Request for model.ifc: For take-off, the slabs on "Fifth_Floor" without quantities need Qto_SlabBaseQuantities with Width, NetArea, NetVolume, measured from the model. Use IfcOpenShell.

First a look at what the model holds.

```python
import ifcopenshell
import ifcopenshell.util.element
import ifcopenshell.util.unit

model = ifcopenshell.open("model.ifc")
print(model.schema)
for unit_type in ("LENGTHUNIT", "AREAUNIT", "VOLUMEUNIT"):
    print(unit_type, ifcopenshell.util.unit.calculate_unit_scale(model, unit_type))
storey = next(s for s in model.by_type("IfcBuildingStorey") if s.Name == "Fifth_Floor")
slabs = [e for e in ifcopenshell.util.element.get_decomposition(storey) if e.is_a("IfcSlab")]
for e in sorted(slabs, key=lambda e: e.id()):
    print(e.id(), e.is_a(), e.Name, list(ifcopenshell.util.element.get_psets(e, qtos_only=True)), sep=" | ")
```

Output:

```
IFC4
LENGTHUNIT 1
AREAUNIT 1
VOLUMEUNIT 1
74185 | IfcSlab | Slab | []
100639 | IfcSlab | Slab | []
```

```python
import ifcopenshell
import ifcopenshell.api.pset
import ifcopenshell.geom
import ifcopenshell.util.element
import ifcopenshell.util.shape
import ifcopenshell.util.unit

model = ifcopenshell.open("model.ifc")
unit_scale = ifcopenshell.util.unit.calculate_unit_scale(model)
area_scale = ifcopenshell.util.unit.calculate_unit_scale(model, "AREAUNIT")
volume_scale = ifcopenshell.util.unit.calculate_unit_scale(model, "VOLUMEUNIT")
settings = ifcopenshell.geom.settings()

storey = next(s for s in model.by_type("IfcBuildingStorey") if s.Name == "Fifth_Floor")
slabs = [e for e in ifcopenshell.util.element.get_decomposition(storey) if e.is_a("IfcSlab")]

for e in sorted(slabs, key=lambda e: e.id()):
    if ifcopenshell.util.element.get_psets(e, qtos_only=True, should_inherit=False):
        continue
    # Geometry comes back in metres, in the element's own axes.
    shape = ifcopenshell.geom.create_shape(settings, e)
    values = {
        "Width": ifcopenshell.util.shape.get_z(shape.geometry) / unit_scale,
        "NetArea": ifcopenshell.util.shape.get_footprint_area(shape.geometry) / area_scale,
        "NetVolume": ifcopenshell.util.shape.get_volume(shape.geometry) / volume_scale,
    }
    qto = ifcopenshell.api.pset.add_qto(model, product=e, name="Qto_SlabBaseQuantities")
    ifcopenshell.api.pset.edit_qto(model, qto=qto, properties=values)
    print(e.id(), {k: round(v, 3) for k, v in values.items()})

model.write("model_updated.ifc")
```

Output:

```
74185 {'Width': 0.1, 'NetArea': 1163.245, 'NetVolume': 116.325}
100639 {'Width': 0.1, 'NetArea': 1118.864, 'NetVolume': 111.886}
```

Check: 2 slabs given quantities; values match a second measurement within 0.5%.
